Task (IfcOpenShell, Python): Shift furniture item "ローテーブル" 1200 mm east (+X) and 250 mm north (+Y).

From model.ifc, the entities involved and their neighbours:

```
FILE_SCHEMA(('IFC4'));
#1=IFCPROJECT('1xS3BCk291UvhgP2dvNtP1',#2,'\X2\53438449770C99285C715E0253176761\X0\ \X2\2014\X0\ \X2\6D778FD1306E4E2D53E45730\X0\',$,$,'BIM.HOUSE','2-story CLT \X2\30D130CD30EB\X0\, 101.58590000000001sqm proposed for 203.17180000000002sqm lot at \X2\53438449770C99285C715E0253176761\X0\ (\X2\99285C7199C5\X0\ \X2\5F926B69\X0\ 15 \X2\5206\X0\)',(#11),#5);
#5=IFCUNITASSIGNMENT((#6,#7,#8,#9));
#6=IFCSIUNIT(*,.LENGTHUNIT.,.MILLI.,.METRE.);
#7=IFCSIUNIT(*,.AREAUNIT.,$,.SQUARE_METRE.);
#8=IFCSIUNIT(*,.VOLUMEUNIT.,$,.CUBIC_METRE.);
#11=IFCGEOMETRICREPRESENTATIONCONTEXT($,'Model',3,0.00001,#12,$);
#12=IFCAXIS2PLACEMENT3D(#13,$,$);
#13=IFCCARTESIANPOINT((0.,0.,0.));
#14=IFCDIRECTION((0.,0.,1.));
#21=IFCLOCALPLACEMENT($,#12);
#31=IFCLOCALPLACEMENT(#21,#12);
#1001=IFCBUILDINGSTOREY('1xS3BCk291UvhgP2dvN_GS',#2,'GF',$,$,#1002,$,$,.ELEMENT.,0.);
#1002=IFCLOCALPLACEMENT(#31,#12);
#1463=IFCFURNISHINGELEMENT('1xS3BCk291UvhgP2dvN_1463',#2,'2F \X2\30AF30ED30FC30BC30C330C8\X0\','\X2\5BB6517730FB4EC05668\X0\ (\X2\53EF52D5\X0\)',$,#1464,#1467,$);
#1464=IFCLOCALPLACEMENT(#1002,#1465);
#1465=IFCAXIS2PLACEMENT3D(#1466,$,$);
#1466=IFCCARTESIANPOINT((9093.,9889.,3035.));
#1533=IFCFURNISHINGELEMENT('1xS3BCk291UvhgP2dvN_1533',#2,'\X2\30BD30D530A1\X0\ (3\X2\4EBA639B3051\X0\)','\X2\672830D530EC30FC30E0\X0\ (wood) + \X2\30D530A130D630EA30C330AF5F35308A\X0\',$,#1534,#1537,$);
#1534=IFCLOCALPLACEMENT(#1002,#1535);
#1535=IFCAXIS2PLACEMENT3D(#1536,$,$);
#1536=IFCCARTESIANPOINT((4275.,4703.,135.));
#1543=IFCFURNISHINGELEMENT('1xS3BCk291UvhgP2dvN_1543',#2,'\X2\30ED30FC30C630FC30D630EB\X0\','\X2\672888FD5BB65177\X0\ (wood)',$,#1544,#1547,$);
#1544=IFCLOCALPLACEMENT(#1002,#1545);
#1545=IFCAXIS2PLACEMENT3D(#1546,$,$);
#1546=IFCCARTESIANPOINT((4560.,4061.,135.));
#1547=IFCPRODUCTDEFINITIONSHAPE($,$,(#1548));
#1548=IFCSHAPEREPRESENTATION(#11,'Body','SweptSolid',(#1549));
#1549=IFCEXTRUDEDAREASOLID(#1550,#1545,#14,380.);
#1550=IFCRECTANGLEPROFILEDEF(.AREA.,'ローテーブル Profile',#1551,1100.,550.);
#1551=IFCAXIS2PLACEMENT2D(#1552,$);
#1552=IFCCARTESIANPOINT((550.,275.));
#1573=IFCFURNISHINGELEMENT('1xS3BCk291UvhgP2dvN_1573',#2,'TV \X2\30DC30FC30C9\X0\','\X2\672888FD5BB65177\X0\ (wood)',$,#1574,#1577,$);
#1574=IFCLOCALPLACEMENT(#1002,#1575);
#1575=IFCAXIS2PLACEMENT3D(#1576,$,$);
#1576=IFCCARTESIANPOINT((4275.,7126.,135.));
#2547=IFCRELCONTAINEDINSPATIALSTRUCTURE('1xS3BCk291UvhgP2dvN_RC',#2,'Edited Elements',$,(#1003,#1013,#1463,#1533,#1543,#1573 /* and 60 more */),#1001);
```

```python
import ifcopenshell
import ifcopenshell.api.geometry
import ifcopenshell.util.placement

model = ifcopenshell.open("model.ifc")

item = model.by_id(1543)
matrix = ifcopenshell.util.placement.get_local_placement(item.ObjectPlacement)
matrix[0, 3] += 1200.0
matrix[1, 3] += 250.0
ifcopenshell.api.geometry.edit_object_placement(model, product=item, matrix=matrix, is_si=False)

print(ifcopenshell.util.placement.get_local_placement(item.ObjectPlacement).round(3) + 0.0)

model.write("model_rev.ifc")
```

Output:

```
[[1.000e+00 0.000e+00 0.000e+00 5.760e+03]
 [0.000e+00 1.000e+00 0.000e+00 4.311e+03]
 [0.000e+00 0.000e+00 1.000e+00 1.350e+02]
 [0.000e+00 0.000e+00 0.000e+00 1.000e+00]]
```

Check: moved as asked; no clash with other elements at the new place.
